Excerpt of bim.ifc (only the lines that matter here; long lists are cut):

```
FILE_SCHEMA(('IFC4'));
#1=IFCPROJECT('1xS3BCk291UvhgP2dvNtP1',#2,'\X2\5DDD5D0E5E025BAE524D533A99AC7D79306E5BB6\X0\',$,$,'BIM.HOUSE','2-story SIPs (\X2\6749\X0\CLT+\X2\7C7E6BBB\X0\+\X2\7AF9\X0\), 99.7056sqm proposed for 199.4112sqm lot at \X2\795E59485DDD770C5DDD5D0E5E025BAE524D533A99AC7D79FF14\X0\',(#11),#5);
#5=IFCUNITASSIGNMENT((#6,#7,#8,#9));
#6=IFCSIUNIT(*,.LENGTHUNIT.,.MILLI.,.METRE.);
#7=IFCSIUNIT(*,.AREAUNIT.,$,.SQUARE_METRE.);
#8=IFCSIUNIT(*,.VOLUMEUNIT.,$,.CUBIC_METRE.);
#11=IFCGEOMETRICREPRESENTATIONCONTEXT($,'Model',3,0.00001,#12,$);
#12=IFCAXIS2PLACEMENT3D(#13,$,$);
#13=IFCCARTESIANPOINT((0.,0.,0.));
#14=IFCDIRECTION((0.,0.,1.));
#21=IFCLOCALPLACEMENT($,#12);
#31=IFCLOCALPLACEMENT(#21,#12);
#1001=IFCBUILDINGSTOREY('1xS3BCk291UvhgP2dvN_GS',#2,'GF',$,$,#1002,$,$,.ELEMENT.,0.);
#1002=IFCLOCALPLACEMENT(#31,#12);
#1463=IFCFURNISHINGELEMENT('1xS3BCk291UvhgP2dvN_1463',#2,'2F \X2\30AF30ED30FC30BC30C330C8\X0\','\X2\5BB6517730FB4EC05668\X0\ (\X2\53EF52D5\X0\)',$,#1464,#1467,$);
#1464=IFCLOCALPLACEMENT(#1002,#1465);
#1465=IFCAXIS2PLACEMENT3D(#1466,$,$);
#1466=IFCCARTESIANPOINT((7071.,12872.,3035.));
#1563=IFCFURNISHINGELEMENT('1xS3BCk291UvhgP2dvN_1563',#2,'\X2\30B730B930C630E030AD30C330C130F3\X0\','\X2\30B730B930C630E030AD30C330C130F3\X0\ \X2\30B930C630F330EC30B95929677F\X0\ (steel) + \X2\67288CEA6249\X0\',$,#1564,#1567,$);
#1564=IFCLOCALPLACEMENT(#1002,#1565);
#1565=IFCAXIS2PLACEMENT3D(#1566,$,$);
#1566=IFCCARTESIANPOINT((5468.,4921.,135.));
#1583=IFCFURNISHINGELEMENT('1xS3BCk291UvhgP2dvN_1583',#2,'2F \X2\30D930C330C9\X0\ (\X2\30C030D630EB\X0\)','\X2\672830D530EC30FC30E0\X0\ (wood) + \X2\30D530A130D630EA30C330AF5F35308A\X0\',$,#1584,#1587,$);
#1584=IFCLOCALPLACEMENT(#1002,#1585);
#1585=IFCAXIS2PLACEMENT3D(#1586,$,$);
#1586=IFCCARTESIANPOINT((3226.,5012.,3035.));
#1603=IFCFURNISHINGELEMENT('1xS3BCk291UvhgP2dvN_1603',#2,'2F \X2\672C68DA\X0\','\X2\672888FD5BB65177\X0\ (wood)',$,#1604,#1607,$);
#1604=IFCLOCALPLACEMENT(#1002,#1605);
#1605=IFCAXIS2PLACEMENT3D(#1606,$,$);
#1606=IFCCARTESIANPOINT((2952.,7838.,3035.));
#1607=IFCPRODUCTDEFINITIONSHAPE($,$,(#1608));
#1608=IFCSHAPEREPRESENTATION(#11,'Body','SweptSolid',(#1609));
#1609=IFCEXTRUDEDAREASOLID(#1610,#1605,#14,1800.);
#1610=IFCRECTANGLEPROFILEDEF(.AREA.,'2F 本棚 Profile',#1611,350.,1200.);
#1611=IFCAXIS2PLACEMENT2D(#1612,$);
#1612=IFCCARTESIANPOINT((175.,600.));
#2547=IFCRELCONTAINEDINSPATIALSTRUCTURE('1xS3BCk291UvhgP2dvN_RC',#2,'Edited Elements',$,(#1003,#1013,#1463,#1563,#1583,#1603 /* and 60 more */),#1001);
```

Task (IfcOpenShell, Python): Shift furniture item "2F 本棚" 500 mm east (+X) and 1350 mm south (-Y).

```python
import ifcopenshell
import ifcopenshell.api.geometry
import ifcopenshell.util.placement
import ifcopenshell.util.unit

model = ifcopenshell.open("bim.ifc")
unit_scale = ifcopenshell.util.unit.calculate_unit_scale(model)

item = model.by_guid("1xS3BCk291UvhgP2dvN_1603")
matrix = ifcopenshell.util.placement.get_local_placement(item.ObjectPlacement)
matrix[0, 3] += 0.5 / unit_scale
matrix[1, 3] -= 1.35 / unit_scale
ifcopenshell.api.geometry.edit_object_placement(model, product=item, matrix=matrix, is_si=False)

print(ifcopenshell.util.placement.get_local_placement(item.ObjectPlacement).round(3) + 0.0)

model.write("bim_rev.ifc")
```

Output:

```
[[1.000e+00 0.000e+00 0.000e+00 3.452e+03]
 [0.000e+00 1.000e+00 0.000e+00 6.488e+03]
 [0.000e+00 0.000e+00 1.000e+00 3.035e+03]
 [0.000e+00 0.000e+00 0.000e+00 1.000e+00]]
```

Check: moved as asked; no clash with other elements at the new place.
